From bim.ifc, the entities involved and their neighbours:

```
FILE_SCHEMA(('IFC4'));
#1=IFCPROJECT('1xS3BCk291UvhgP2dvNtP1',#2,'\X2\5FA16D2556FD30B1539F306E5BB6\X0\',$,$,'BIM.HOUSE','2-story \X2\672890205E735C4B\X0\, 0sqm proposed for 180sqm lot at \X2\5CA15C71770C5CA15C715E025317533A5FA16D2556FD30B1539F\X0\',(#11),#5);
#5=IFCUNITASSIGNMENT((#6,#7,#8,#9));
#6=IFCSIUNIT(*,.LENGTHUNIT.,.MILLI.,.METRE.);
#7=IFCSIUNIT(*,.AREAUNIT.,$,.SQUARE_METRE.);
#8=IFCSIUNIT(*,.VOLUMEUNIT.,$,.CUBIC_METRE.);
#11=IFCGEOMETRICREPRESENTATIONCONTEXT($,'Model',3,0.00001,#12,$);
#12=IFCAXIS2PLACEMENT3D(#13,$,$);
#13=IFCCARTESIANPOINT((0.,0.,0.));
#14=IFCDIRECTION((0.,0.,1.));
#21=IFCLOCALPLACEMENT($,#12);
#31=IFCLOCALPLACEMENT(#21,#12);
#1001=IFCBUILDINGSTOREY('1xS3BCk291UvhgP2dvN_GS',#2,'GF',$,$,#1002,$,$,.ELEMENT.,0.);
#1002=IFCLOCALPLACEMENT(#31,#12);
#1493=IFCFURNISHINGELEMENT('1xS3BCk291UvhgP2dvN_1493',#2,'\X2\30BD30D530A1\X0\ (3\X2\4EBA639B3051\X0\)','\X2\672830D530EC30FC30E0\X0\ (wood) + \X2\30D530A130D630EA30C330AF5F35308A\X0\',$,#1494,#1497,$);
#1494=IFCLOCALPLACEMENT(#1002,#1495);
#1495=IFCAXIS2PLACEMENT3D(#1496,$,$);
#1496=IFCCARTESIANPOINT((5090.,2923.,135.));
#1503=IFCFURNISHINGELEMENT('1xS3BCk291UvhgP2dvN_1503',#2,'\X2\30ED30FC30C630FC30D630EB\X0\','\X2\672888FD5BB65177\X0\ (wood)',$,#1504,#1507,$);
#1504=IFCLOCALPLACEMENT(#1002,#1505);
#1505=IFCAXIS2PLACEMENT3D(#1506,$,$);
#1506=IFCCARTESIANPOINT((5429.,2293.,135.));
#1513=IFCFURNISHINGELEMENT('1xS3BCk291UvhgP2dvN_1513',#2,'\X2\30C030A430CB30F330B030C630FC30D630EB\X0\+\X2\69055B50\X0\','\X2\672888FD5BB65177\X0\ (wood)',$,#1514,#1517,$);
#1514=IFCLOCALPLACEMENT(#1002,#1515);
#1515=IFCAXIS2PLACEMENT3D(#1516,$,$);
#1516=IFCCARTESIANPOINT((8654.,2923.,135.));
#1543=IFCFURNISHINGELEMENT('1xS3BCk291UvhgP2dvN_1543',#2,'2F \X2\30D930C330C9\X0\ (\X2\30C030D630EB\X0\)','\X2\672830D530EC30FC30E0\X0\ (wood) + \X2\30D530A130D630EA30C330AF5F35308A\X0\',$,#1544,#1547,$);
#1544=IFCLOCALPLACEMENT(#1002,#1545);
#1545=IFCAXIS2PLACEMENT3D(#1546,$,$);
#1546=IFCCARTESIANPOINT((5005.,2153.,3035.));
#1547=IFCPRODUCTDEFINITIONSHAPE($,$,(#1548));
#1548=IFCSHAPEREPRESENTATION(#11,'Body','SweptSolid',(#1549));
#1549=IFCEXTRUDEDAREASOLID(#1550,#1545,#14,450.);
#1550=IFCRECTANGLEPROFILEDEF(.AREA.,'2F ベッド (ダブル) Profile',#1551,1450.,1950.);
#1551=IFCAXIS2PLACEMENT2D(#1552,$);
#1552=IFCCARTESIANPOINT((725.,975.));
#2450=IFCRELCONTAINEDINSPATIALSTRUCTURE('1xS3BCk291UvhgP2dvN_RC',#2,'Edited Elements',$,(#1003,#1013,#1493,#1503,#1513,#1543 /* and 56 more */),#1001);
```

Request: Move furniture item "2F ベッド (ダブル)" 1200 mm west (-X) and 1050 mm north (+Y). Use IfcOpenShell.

```python
import ifcopenshell
import ifcopenshell.api.geometry
import ifcopenshell.util.placement
import ifcopenshell.util.unit

model = ifcopenshell.open("bim.ifc")
unit_scale = ifcopenshell.util.unit.calculate_unit_scale(model)

item = model.by_guid("1xS3BCk291UvhgP2dvN_1543")
matrix = ifcopenshell.util.placement.get_local_placement(item.ObjectPlacement)
matrix[0, 3] -= 1.2 / unit_scale
matrix[1, 3] += 1.05 / unit_scale
ifcopenshell.api.geometry.edit_object_placement(model, product=item, matrix=matrix, is_si=False)

print(ifcopenshell.util.placement.get_local_placement(item.ObjectPlacement).round(3) + 0.0)

model.write("bim-out.ifc")
```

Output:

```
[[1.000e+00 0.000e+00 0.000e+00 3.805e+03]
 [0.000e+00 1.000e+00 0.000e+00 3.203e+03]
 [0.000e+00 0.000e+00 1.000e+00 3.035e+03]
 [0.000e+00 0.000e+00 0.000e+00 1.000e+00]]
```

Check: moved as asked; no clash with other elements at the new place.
